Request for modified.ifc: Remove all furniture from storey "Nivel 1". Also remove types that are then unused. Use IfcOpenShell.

First a look at what the model holds.

```python
import ifcopenshell
import ifcopenshell.util.element

model = ifcopenshell.open("modified.ifc")
print(model.schema)
storey = next(s for s in model.by_type("IfcBuildingStorey") if s.Name == "Nivel 1")
furniture = [e for e in ifcopenshell.util.element.get_decomposition(storey) if e.is_a("IfcFurnishingElement")]
seen = {}
for e in furniture:
    element_type = ifcopenshell.util.element.get_type(e)
    name = element_type.Name if element_type not in (None, e) else None
    seen[name] = seen.get(name, 0) + 1
for name, count in sorted(seen.items(), key=str):
    print(count, "x", name)
```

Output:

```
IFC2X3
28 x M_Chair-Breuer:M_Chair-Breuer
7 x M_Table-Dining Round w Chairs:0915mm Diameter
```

```python
import ifcopenshell
import ifcopenshell.api.root
import ifcopenshell.util.element

model = ifcopenshell.open("modified.ifc")

storey = next(s for s in model.by_type("IfcBuildingStorey") if s.Name == "Nivel 1")
furniture = [e for e in ifcopenshell.util.element.get_decomposition(storey) if e.is_a("IfcFurnishingElement")]
types = {ifcopenshell.util.element.get_type(e) for e in furniture} - {None, *furniture}

for e in furniture:
    ifcopenshell.api.root.remove_product(model, product=e)
print(len(furniture), "removed")

unused = [t for t in types if not ifcopenshell.util.element.get_types(t)]
for t in unused:
    ifcopenshell.api.root.remove_product(model, product=t)
print(len(unused), "unused types removed")

model.write("modified_edited.ifc")
```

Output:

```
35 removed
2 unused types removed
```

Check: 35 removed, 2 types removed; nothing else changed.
